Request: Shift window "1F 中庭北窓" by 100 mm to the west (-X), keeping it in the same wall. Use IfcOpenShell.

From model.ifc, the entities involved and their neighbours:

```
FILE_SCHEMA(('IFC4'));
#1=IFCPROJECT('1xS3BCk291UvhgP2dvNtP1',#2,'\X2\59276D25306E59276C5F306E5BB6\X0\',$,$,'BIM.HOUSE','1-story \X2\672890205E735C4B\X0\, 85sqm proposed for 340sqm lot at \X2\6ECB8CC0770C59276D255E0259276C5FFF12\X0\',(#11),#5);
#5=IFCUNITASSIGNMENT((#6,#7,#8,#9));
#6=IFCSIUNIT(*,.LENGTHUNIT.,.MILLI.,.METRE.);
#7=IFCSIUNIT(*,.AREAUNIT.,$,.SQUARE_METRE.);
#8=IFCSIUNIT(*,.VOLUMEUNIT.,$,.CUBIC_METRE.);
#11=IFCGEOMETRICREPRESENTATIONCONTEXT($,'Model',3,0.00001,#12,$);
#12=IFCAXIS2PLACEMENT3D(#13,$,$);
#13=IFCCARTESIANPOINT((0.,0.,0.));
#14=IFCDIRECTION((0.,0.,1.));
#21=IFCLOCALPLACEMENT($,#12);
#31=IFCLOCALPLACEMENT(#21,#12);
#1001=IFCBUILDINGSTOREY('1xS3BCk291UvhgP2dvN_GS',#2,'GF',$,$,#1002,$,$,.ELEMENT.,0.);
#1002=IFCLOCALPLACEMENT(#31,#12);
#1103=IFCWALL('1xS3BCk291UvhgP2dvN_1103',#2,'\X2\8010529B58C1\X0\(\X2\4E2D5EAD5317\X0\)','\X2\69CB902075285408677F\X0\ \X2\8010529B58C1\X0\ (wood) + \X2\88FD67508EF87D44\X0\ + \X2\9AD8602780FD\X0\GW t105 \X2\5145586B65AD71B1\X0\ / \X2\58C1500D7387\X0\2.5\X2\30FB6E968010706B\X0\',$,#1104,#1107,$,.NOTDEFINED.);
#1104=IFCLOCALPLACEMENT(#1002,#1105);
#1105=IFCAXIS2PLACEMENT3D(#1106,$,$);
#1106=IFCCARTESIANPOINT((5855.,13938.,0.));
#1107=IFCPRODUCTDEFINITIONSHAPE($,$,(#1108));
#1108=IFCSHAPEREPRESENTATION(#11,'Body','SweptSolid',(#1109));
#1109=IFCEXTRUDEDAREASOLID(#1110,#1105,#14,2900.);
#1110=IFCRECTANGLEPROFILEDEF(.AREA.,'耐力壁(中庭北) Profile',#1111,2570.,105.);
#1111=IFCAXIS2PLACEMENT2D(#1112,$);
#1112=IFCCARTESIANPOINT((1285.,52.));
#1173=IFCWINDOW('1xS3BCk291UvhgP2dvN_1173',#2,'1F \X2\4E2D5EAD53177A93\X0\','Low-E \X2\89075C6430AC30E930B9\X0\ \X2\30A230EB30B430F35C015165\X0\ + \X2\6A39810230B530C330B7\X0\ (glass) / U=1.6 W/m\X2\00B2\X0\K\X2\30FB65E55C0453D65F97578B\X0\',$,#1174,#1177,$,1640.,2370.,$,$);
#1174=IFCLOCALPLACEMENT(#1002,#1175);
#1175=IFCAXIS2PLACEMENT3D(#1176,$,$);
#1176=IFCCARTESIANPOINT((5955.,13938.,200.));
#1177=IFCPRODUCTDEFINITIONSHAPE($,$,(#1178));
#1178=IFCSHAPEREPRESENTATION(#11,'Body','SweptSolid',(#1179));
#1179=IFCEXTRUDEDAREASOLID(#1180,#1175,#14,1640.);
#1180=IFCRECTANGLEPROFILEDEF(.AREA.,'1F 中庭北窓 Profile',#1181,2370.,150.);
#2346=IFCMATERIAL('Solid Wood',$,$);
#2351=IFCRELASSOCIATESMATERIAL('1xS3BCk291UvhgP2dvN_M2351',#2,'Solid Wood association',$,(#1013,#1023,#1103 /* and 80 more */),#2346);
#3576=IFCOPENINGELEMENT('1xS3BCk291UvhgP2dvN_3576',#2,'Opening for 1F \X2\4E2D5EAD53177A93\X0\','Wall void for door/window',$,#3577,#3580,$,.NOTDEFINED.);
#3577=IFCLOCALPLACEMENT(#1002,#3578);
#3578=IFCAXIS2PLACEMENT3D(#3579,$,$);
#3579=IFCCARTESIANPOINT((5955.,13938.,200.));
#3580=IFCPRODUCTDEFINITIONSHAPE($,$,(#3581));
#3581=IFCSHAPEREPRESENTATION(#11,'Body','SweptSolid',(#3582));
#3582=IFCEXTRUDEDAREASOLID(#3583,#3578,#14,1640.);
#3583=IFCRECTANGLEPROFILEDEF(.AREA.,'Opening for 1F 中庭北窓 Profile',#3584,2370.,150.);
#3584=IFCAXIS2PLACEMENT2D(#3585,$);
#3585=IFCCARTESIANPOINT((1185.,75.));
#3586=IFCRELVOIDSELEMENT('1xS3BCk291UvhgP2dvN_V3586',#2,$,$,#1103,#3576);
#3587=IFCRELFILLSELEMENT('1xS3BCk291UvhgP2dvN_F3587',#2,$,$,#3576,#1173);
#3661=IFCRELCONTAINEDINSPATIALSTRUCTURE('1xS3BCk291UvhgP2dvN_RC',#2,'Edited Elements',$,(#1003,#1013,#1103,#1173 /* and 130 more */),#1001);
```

```python
import ifcopenshell
import ifcopenshell.api.geometry
import ifcopenshell.util.placement

model = ifcopenshell.open("model.ifc")

window = model.by_id(1173)
opening = window.FillsVoids[0].RelatingOpeningElement
wall = opening.VoidsElements[0].RelatingBuildingElement

wall_matrix = ifcopenshell.util.placement.get_local_placement(wall.ObjectPlacement)
shift = wall_matrix[:3, 0] * -100.0
before = ifcopenshell.util.placement.get_local_placement(window.ObjectPlacement)[:3, 3].copy()

# The window is not placed relative to its opening, so move both.
for product in (opening, window):
    matrix = ifcopenshell.util.placement.get_local_placement(product.ObjectPlacement)
    matrix[:3, 3] += shift
    ifcopenshell.api.geometry.edit_object_placement(model, product=product, matrix=matrix, is_si=False)

after = ifcopenshell.util.placement.get_local_placement(window.ObjectPlacement)[:3, 3]
print("window moved by", (after - before).round(3) + 0.0)

model.write("model_edited.ifc")
```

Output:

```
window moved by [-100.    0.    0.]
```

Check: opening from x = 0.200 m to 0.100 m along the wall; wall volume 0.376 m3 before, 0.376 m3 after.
